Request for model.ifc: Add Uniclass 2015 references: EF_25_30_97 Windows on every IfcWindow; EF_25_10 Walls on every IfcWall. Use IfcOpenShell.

First a look at what the model holds.

```python
import ifcopenshell

model = ifcopenshell.open("model.ifc")
print(model.schema)
print("classifications:", [c.Name for c in model.by_type("IfcClassification")])
for ifc_class in ("IfcDoor", "IfcRoof", "IfcStair", "IfcWall", "IfcWindow"):
    print(ifc_class, len(model.by_type(ifc_class)))
```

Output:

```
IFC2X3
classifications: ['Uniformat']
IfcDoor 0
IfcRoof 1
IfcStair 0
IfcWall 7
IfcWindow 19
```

```python
import ifcopenshell
import ifcopenshell.api.classification

model = ifcopenshell.open("model.ifc")

# IFC2X3 requires Source and Edition and has no link from the project to the system.
system = model.create_entity("IfcClassification", Source="NBS", Edition="2015", Name="Uniclass 2015")

codes = {
    "IfcWindow": ("EF_25_30_97", "Windows"),
    "IfcWall": ("EF_25_10", "Walls"),
}
for ifc_class, (code, name) in codes.items():
    products = model.by_type(ifc_class)
    ifcopenshell.api.classification.add_reference(
        model, products=products, classification=system, identification=code, name=name
    )
    print(code, len(products))

model.write("model_rev.ifc")
```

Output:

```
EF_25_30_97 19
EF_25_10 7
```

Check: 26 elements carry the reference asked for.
